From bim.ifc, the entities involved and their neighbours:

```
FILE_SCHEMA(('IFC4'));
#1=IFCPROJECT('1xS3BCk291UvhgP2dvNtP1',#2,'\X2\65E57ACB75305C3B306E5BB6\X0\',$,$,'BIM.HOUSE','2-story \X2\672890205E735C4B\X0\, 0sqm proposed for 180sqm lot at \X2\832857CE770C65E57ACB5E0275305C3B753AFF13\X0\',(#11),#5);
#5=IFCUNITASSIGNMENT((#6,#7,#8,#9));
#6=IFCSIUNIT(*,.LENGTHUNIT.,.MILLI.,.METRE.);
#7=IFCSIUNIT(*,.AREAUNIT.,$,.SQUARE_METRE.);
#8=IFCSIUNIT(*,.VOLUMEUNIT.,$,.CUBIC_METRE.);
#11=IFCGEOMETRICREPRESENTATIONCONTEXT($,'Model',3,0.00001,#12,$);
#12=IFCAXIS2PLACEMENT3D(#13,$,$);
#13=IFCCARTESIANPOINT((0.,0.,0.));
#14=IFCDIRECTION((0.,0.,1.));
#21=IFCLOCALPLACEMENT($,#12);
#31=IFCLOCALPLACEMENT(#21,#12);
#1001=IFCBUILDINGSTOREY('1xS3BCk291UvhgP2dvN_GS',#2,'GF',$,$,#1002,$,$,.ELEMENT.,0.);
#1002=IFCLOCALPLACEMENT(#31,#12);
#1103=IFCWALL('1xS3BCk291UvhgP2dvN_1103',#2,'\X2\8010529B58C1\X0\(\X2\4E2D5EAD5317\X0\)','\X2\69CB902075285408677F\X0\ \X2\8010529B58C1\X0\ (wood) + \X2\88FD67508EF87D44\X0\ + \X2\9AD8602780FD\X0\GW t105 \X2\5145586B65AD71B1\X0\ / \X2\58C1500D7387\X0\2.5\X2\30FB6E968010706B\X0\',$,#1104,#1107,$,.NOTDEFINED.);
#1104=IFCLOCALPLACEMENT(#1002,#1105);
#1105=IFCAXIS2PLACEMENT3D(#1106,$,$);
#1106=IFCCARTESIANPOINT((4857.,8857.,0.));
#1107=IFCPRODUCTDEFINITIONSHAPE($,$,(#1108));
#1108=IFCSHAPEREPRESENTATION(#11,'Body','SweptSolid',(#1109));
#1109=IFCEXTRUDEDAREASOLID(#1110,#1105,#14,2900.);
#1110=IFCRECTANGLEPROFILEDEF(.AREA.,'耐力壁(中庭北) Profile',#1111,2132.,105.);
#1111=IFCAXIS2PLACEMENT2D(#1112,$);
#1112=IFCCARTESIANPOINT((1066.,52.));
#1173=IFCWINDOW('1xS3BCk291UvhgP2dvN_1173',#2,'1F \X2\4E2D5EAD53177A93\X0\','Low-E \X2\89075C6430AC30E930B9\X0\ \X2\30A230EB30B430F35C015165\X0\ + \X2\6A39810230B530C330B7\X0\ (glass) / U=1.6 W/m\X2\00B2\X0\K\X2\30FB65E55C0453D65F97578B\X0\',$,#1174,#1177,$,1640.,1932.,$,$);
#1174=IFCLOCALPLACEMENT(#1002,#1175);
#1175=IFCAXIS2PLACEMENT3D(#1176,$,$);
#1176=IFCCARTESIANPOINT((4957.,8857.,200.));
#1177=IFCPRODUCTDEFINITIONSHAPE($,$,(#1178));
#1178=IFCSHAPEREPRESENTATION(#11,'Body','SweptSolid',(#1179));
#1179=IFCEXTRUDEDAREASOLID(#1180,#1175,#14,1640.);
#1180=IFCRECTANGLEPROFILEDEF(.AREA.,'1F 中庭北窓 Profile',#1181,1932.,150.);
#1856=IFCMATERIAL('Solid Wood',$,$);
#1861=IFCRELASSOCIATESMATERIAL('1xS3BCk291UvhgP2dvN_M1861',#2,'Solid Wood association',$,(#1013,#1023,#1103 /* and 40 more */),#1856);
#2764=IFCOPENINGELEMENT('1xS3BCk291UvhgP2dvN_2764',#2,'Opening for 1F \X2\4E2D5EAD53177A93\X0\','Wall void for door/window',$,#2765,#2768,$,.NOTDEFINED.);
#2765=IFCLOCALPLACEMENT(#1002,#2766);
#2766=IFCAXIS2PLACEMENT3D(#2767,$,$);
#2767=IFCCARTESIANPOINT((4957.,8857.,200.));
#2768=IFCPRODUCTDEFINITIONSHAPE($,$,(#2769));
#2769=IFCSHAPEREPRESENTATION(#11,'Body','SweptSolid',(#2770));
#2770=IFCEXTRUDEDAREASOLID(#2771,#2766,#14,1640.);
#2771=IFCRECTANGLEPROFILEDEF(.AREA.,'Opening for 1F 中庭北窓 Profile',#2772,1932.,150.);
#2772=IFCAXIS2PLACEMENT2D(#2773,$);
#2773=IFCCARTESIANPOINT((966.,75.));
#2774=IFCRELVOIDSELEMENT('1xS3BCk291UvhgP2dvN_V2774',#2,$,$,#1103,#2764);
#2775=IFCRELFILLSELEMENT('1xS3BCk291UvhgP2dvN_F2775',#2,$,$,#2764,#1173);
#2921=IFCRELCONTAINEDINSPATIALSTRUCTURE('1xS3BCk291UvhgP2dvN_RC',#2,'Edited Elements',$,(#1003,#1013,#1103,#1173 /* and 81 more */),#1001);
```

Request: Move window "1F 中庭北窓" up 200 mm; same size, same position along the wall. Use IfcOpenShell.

```python
import numpy as np
import ifcopenshell
import ifcopenshell.api.geometry
import ifcopenshell.util.placement
import ifcopenshell.util.unit

model = ifcopenshell.open("bim.ifc")
unit_scale = ifcopenshell.util.unit.calculate_unit_scale(model)

window = model.by_guid("1xS3BCk291UvhgP2dvN_1173")
opening = window.FillsVoids[0].RelatingOpeningElement
dz = 0.2 / unit_scale

shift = np.array([0.0, 0.0, dz])
# The window is not placed relative to its opening, so move both.
for product in (opening, window):
    matrix = ifcopenshell.util.placement.get_local_placement(product.ObjectPlacement)
    matrix[:3, 3] += shift
    ifcopenshell.api.geometry.edit_object_placement(model, product=product, matrix=matrix, is_si=False)

print(f"moved by {dz * unit_scale:+.3f} m")

model.write("bim-out.ifc")
```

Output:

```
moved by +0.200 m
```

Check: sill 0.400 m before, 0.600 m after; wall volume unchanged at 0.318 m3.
